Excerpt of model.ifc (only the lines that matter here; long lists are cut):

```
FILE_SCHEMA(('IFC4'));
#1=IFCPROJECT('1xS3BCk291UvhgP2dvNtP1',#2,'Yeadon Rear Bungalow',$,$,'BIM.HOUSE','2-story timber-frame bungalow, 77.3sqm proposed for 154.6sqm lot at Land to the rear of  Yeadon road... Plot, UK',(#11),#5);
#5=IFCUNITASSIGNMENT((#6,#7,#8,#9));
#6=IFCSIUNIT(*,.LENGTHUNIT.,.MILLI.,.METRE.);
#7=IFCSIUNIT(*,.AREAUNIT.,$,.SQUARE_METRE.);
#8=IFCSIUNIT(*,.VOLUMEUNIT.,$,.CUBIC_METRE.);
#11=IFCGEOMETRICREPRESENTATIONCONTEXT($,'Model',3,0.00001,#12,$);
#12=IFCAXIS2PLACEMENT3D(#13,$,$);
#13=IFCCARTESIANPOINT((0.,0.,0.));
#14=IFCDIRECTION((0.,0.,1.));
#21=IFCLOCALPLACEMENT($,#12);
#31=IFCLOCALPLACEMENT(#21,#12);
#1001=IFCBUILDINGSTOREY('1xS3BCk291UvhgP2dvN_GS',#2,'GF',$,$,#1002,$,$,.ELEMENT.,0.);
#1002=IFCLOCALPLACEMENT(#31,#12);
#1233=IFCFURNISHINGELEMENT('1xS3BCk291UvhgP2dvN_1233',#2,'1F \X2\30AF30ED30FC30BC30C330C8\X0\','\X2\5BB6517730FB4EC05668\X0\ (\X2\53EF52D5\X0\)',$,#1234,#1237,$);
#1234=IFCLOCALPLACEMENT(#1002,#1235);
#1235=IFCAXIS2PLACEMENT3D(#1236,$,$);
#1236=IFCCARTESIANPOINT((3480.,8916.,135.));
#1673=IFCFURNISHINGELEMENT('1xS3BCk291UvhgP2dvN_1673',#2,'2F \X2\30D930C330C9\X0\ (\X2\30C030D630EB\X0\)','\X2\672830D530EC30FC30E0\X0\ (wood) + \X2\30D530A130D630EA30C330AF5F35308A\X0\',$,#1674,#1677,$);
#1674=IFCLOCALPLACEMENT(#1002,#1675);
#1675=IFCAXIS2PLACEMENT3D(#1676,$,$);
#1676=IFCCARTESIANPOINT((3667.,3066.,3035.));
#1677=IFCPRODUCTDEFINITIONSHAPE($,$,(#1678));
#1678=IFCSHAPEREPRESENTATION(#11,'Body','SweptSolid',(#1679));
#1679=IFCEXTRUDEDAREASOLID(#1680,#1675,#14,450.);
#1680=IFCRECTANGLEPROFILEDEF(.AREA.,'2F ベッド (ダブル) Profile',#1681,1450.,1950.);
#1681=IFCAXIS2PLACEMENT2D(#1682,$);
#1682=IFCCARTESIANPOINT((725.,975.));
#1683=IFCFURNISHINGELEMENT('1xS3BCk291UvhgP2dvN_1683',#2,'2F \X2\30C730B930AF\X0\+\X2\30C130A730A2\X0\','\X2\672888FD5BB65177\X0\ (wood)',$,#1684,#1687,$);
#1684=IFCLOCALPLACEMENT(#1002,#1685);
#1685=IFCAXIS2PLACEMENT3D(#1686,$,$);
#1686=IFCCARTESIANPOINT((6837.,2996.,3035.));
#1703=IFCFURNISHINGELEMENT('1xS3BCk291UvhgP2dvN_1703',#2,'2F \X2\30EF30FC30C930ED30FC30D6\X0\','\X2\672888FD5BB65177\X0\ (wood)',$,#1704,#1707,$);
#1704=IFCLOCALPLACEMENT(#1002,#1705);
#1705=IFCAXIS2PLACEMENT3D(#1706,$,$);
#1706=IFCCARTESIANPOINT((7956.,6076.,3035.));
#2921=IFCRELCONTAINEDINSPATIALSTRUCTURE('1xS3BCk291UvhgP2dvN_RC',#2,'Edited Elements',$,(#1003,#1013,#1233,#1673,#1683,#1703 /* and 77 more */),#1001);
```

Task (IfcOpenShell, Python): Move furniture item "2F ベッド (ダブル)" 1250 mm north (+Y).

```python
import ifcopenshell
import ifcopenshell.api.geometry
import ifcopenshell.util.placement
import ifcopenshell.util.unit

model = ifcopenshell.open("model.ifc")
unit_scale = ifcopenshell.util.unit.calculate_unit_scale(model)

item = model.by_guid("1xS3BCk291UvhgP2dvN_1673")
matrix = ifcopenshell.util.placement.get_local_placement(item.ObjectPlacement)
matrix[1, 3] += 1.25 / unit_scale
ifcopenshell.api.geometry.edit_object_placement(model, product=item, matrix=matrix, is_si=False)

print(ifcopenshell.util.placement.get_local_placement(item.ObjectPlacement).round(3) + 0.0)

model.write("model-out.ifc")
```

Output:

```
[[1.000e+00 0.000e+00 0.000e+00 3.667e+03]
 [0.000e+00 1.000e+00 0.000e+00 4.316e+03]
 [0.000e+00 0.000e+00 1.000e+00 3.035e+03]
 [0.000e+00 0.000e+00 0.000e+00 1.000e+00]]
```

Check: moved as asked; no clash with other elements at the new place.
